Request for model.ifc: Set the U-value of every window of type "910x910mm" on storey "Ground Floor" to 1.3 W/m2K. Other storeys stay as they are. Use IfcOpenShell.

First a look at what the model holds.

```python
import ifcopenshell
import ifcopenshell.util.element

model = ifcopenshell.open("model.ifc")
print(model.schema)
storey = next(s for s in model.by_type("IfcBuildingStorey") if s.Name == "Ground Floor")
windows = [e for e in ifcopenshell.util.element.get_decomposition(storey) if e.is_a("IfcWindow")]
seen = {}
for e in windows:
    element_type = ifcopenshell.util.element.get_type(e)
    key = (element_type.Name if element_type != e and element_type else None, ifcopenshell.util.element.get_pset(e, "Pset_WindowCommon", "ThermalTransmittance"))
    seen[key] = seen.get(key, 0) + 1
for (name, value), count in sorted(seen.items(), key=str):
    print(count, "x", name, "|", value)
```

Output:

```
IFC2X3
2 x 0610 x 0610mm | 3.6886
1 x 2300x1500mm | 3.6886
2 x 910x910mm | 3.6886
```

```python
import ifcopenshell
import ifcopenshell.api.pset
import ifcopenshell.util.element

model = ifcopenshell.open("model.ifc")

storey = next(s for s in model.by_type("IfcBuildingStorey") if s.Name == "Ground Floor")
windows = [e for e in ifcopenshell.util.element.get_decomposition(storey) if e.is_a("IfcWindow")]

count = 0
for e in windows:
    element_type = ifcopenshell.util.element.get_type(e)
    if element_type in (None, e) or element_type.Name != "910x910mm":
        continue
    # add_pset returns the element's existing set when there is one.
    pset = ifcopenshell.api.pset.add_pset(model, product=e, name="Pset_WindowCommon")
    ifcopenshell.api.pset.edit_pset(model, pset=pset, properties={"ThermalTransmittance": 1.3})
    count += 1

print(count, "windows updated")

model.write("model_rev.ifc")
```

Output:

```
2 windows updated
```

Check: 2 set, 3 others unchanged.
